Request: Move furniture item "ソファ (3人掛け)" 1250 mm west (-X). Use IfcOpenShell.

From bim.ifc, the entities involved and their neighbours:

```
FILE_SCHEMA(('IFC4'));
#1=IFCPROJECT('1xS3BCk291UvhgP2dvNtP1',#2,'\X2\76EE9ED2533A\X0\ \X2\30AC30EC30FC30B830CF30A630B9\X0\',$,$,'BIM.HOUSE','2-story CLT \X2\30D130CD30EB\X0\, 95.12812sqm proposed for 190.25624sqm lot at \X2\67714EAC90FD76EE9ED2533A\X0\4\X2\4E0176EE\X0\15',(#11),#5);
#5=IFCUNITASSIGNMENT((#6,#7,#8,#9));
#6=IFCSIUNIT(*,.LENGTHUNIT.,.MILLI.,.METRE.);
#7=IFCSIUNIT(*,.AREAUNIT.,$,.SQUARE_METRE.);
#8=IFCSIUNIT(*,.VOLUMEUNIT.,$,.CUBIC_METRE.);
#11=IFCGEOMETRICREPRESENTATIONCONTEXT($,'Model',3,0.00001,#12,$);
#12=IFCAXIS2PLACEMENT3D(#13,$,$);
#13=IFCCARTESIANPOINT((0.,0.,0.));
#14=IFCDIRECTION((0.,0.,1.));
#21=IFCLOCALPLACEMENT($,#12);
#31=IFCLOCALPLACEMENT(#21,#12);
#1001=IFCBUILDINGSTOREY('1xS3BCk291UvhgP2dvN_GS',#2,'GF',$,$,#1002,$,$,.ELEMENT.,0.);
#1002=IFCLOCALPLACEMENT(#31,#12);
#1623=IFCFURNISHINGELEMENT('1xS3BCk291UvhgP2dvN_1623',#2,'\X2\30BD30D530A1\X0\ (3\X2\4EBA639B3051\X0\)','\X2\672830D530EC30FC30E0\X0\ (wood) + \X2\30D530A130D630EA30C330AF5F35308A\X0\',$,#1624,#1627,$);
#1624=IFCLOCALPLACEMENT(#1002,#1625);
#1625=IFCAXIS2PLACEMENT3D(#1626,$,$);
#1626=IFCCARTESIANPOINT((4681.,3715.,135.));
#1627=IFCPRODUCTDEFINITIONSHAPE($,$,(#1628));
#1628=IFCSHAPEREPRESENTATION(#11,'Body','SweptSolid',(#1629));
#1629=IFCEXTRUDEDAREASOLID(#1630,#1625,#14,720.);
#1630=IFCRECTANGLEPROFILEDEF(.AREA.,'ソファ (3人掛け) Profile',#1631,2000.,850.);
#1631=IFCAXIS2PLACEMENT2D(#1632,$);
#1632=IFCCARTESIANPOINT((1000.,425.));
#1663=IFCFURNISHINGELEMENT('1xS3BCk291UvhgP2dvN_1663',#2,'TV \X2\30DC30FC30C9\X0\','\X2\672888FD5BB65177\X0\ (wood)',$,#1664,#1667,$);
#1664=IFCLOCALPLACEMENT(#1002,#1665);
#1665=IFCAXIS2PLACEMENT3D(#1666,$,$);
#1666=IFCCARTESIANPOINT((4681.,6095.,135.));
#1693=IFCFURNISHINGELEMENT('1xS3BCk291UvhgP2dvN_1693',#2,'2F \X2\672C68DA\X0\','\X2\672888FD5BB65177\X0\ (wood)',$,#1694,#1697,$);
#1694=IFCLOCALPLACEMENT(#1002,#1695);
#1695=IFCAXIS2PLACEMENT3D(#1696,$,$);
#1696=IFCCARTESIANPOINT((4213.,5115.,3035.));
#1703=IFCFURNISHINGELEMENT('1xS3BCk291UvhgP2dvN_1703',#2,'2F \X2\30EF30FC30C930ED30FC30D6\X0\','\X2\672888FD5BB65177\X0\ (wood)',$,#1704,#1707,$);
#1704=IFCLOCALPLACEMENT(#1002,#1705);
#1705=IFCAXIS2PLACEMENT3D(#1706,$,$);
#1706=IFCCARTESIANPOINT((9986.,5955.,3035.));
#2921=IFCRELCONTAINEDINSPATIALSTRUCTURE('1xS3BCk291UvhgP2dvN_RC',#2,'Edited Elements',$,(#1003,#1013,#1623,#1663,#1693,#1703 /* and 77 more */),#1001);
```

```python
import ifcopenshell
import ifcopenshell.api.geometry
import ifcopenshell.util.placement
import ifcopenshell.util.unit

model = ifcopenshell.open("bim.ifc")
unit_scale = ifcopenshell.util.unit.calculate_unit_scale(model)

item = model.by_id(1623)
matrix = ifcopenshell.util.placement.get_local_placement(item.ObjectPlacement)
matrix[0, 3] -= 1.25 / unit_scale
ifcopenshell.api.geometry.edit_object_placement(model, product=item, matrix=matrix, is_si=False)

print(ifcopenshell.util.placement.get_local_placement(item.ObjectPlacement).round(3) + 0.0)

model.write("bim-out.ifc")
```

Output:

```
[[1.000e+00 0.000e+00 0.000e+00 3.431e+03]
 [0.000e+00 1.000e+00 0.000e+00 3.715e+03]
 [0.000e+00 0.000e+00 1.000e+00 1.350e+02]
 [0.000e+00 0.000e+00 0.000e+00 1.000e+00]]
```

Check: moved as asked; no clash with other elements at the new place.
